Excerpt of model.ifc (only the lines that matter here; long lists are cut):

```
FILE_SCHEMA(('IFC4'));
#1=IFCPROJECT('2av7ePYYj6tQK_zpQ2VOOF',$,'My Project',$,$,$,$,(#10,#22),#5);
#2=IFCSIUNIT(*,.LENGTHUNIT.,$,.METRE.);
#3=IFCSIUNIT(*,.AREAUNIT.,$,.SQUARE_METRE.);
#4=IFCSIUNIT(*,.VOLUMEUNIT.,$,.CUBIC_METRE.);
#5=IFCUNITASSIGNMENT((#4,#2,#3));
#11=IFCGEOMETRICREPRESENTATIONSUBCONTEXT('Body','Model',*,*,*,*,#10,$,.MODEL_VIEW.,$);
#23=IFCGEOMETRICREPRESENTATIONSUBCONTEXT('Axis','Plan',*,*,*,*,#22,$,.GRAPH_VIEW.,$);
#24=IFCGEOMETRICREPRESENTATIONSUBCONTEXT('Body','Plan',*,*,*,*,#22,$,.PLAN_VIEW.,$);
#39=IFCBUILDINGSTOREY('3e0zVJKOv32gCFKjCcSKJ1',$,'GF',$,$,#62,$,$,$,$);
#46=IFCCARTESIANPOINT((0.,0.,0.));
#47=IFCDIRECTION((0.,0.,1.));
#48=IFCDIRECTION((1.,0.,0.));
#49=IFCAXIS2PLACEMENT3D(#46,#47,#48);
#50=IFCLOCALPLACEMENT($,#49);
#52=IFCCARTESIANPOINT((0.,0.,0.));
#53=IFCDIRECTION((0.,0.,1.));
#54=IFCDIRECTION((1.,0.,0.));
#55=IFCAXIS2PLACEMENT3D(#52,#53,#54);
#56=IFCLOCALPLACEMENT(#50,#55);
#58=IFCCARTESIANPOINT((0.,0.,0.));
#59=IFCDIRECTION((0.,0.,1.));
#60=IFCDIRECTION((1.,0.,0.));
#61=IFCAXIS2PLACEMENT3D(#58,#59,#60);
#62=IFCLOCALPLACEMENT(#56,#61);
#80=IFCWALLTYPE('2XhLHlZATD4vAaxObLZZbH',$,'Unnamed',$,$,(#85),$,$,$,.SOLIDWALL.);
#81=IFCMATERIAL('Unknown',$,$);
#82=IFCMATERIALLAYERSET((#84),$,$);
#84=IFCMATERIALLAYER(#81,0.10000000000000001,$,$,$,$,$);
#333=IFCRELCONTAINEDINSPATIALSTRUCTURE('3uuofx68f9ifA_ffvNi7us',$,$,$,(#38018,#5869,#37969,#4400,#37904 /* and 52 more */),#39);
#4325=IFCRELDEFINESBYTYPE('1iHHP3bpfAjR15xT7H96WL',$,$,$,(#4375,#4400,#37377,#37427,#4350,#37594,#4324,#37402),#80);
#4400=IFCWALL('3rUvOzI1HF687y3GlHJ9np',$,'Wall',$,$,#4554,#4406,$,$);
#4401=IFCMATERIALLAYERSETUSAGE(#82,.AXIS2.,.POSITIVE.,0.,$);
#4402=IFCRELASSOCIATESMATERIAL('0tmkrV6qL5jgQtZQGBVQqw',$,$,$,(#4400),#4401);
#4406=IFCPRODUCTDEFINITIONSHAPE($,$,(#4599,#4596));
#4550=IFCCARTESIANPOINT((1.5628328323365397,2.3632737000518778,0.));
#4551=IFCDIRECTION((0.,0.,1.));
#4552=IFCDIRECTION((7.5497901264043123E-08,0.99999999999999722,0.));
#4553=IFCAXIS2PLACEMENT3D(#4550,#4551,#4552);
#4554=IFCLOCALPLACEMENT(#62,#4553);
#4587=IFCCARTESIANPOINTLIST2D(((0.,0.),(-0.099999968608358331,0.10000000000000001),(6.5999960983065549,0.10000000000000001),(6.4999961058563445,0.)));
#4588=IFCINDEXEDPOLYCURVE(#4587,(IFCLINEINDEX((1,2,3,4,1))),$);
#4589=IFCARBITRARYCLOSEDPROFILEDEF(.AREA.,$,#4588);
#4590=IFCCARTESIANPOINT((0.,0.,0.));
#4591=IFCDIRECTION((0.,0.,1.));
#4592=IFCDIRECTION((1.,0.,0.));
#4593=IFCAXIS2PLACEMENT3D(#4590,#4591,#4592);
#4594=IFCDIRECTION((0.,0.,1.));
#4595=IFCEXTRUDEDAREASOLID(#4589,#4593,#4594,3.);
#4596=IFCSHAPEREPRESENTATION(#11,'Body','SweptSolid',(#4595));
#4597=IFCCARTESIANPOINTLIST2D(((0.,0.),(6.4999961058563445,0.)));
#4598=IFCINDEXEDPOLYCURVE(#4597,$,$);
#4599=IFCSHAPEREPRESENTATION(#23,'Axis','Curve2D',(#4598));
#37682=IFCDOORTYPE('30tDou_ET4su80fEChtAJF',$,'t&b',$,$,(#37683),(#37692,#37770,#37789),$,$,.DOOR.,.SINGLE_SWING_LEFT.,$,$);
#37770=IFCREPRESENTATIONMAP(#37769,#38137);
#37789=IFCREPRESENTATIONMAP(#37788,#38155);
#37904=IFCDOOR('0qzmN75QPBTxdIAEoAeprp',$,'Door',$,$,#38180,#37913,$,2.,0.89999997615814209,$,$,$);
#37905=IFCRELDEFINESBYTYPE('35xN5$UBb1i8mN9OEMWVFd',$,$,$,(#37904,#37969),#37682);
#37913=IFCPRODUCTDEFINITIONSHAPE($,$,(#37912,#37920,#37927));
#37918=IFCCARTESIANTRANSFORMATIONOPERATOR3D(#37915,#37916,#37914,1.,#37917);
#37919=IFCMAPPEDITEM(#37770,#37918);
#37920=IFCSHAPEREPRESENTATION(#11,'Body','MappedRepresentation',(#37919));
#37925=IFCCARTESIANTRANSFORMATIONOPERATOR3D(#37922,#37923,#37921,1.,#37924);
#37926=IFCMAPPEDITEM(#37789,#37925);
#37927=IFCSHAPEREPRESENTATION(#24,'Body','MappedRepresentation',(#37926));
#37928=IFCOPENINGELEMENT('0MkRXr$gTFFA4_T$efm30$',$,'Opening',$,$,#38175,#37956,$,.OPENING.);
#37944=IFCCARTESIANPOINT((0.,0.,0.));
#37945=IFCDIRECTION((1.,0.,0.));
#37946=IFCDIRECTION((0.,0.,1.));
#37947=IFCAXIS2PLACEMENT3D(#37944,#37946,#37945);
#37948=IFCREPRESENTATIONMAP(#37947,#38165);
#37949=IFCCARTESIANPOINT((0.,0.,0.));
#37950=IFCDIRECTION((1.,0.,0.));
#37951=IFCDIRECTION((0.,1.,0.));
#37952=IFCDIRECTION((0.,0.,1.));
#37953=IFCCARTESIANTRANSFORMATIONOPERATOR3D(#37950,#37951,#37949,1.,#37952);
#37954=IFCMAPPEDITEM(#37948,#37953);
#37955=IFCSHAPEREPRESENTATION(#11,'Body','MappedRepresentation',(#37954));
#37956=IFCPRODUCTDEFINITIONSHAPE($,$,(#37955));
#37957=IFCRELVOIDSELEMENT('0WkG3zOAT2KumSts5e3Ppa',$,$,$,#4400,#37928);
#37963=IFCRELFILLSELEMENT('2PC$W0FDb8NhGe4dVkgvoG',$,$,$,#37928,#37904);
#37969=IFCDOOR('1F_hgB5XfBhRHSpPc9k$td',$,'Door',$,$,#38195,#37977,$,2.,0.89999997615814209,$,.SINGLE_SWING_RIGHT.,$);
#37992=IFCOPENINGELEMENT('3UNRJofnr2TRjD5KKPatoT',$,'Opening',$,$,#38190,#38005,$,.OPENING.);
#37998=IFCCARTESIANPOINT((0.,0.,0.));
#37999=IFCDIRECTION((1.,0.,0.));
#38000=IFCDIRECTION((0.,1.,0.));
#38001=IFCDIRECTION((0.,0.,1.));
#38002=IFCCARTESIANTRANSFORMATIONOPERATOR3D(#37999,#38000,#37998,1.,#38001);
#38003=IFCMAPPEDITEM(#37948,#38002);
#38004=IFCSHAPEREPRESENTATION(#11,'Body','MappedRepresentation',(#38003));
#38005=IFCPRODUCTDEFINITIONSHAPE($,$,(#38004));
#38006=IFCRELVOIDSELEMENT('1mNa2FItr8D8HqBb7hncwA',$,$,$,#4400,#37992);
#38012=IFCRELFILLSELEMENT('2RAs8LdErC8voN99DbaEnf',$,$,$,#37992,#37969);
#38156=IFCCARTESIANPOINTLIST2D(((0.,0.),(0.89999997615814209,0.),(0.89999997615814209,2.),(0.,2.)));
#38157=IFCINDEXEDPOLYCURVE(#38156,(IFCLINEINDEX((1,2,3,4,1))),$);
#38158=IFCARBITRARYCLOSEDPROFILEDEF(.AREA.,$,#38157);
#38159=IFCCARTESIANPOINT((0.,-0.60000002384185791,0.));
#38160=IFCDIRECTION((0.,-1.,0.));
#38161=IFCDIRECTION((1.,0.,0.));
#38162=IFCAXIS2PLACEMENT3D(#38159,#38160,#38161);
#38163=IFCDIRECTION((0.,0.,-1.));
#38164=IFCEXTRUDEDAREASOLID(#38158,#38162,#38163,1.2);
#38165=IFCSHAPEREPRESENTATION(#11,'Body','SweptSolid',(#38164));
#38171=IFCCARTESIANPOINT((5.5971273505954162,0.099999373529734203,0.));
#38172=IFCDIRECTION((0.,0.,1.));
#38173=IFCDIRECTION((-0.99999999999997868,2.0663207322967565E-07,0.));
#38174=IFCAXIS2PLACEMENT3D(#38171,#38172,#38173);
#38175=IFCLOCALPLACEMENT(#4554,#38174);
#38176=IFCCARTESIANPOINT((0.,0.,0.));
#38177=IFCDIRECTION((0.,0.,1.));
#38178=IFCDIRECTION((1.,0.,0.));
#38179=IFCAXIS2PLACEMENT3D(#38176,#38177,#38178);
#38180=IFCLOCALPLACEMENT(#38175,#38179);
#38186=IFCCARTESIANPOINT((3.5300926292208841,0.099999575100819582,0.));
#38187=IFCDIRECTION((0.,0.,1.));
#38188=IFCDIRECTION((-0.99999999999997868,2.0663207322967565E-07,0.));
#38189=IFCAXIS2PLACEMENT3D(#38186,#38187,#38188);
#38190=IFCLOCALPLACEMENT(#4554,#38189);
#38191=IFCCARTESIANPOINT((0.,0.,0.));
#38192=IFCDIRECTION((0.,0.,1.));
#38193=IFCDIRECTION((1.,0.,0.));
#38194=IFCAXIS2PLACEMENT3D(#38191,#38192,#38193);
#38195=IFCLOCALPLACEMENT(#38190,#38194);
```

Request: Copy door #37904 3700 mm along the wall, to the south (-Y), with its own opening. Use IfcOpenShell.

```python
import ifcopenshell
import ifcopenshell.api.feature
import ifcopenshell.api.geometry
import ifcopenshell.api.root
import ifcopenshell.geom
import ifcopenshell.util.element
import ifcopenshell.util.placement
import ifcopenshell.util.shape
import ifcopenshell.util.unit

model = ifcopenshell.open("model.ifc")
unit_scale = ifcopenshell.util.unit.calculate_unit_scale(model)
settings = ifcopenshell.geom.settings()


def volume(element):
    """Net volume in cubic metres, openings subtracted."""
    shape = ifcopenshell.geom.create_shape(settings, element)
    return ifcopenshell.util.shape.get_volume(shape.geometry)


door = model.by_guid("0qzmN75QPBTxdIAEoAeprp")
opening = door.FillsVoids[0].RelatingOpeningElement
wall = opening.VoidsElements[0].RelatingBuildingElement
before = volume(wall)
shift = ifcopenshell.util.placement.get_local_placement(wall.ObjectPlacement)[:3, 0] * -3.7 / unit_scale

# copy_class copies the void relationship, type, container and properties, but no geometry.
new_opening = ifcopenshell.api.root.copy_class(model, product=opening)
new_opening.Representation = ifcopenshell.util.element.copy_deep(
    model, opening.Representation, exclude=["IfcGeometricRepresentationContext", "IfcRepresentationMap"]
)
new_door = ifcopenshell.api.root.copy_class(model, product=door)
new_door.Representation = ifcopenshell.util.element.copy_deep(
    model, door.Representation, exclude=["IfcGeometricRepresentationContext", "IfcRepresentationMap"]
)
ifcopenshell.api.feature.add_filling(model, opening=new_opening, element=new_door)

for old, new in ((opening, new_opening), (door, new_door)):
    matrix = ifcopenshell.util.placement.get_local_placement(old.ObjectPlacement)
    matrix[:3, 3] += shift
    ifcopenshell.api.geometry.edit_object_placement(model, product=new, matrix=matrix, is_si=False)

after = volume(wall)

print(f"wall volume {before:.3f} -> {after:.3f} m3")

model.write("model_rev.ifc")
```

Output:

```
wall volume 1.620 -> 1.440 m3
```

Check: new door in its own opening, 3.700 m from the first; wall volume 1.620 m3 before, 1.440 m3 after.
